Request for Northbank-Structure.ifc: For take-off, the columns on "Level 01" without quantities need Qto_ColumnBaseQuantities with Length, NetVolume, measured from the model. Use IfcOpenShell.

First a look at what the model holds.

```python
import ifcopenshell
import ifcopenshell.util.element
import ifcopenshell.util.unit

model = ifcopenshell.open("Northbank-Structure.ifc")
print(model.schema)
for unit_type in ("LENGTHUNIT", "AREAUNIT", "VOLUMEUNIT"):
    print(unit_type, ifcopenshell.util.unit.calculate_unit_scale(model, unit_type))
storey = next(s for s in model.by_type("IfcBuildingStorey") if s.Name == "Level 01")
columns = [e for e in ifcopenshell.util.element.get_decomposition(storey) if e.is_a("IfcColumn")]
for e in sorted(columns, key=lambda e: e.id()):
    print(e.id(), e.is_a(), e.Name, list(ifcopenshell.util.element.get_psets(e, qtos_only=True)), sep=" | ")
```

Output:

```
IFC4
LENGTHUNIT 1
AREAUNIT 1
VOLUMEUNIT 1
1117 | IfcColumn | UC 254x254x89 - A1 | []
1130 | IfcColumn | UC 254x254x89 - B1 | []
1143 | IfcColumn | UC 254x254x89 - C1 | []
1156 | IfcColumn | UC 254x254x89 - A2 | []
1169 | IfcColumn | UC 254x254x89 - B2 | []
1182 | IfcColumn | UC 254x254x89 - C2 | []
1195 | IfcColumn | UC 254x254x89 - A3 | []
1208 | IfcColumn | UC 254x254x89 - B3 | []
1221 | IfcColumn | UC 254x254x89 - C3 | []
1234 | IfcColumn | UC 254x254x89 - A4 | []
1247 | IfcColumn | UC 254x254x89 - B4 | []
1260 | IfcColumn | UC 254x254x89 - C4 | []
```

```python
import ifcopenshell
import ifcopenshell.api.pset
import ifcopenshell.geom
import ifcopenshell.util.element
import ifcopenshell.util.shape
import ifcopenshell.util.unit

model = ifcopenshell.open("Northbank-Structure.ifc")
unit_scale = ifcopenshell.util.unit.calculate_unit_scale(model)
volume_scale = ifcopenshell.util.unit.calculate_unit_scale(model, "VOLUMEUNIT")
settings = ifcopenshell.geom.settings()

storey = next(s for s in model.by_type("IfcBuildingStorey") if s.Name == "Level 01")
columns = [e for e in ifcopenshell.util.element.get_decomposition(storey) if e.is_a("IfcColumn")]

for e in sorted(columns, key=lambda e: e.id()):
    if ifcopenshell.util.element.get_psets(e, qtos_only=True, should_inherit=False):
        continue
    # Geometry comes back in metres, in the element's own axes.
    shape = ifcopenshell.geom.create_shape(settings, e)
    values = {
        "Length": ifcopenshell.util.shape.get_z(shape.geometry) / unit_scale,
        "NetVolume": ifcopenshell.util.shape.get_volume(shape.geometry) / volume_scale,
    }
    qto = ifcopenshell.api.pset.add_qto(model, product=e, name="Qto_ColumnBaseQuantities")
    ifcopenshell.api.pset.edit_qto(model, qto=qto, properties=values)
    print(e.id(), {k: round(v, 3) for k, v in values.items()})

model.write("Northbank-Structure_edited.ifc")
```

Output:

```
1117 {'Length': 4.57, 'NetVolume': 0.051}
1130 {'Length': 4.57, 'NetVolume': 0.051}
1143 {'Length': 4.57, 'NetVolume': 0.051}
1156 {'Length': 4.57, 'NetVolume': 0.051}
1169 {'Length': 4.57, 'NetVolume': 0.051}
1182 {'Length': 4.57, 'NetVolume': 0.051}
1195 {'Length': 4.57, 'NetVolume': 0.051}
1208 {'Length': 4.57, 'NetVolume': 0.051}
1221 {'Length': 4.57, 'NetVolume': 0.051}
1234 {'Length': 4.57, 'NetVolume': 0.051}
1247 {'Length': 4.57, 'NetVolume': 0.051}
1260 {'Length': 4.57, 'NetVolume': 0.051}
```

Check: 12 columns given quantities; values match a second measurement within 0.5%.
